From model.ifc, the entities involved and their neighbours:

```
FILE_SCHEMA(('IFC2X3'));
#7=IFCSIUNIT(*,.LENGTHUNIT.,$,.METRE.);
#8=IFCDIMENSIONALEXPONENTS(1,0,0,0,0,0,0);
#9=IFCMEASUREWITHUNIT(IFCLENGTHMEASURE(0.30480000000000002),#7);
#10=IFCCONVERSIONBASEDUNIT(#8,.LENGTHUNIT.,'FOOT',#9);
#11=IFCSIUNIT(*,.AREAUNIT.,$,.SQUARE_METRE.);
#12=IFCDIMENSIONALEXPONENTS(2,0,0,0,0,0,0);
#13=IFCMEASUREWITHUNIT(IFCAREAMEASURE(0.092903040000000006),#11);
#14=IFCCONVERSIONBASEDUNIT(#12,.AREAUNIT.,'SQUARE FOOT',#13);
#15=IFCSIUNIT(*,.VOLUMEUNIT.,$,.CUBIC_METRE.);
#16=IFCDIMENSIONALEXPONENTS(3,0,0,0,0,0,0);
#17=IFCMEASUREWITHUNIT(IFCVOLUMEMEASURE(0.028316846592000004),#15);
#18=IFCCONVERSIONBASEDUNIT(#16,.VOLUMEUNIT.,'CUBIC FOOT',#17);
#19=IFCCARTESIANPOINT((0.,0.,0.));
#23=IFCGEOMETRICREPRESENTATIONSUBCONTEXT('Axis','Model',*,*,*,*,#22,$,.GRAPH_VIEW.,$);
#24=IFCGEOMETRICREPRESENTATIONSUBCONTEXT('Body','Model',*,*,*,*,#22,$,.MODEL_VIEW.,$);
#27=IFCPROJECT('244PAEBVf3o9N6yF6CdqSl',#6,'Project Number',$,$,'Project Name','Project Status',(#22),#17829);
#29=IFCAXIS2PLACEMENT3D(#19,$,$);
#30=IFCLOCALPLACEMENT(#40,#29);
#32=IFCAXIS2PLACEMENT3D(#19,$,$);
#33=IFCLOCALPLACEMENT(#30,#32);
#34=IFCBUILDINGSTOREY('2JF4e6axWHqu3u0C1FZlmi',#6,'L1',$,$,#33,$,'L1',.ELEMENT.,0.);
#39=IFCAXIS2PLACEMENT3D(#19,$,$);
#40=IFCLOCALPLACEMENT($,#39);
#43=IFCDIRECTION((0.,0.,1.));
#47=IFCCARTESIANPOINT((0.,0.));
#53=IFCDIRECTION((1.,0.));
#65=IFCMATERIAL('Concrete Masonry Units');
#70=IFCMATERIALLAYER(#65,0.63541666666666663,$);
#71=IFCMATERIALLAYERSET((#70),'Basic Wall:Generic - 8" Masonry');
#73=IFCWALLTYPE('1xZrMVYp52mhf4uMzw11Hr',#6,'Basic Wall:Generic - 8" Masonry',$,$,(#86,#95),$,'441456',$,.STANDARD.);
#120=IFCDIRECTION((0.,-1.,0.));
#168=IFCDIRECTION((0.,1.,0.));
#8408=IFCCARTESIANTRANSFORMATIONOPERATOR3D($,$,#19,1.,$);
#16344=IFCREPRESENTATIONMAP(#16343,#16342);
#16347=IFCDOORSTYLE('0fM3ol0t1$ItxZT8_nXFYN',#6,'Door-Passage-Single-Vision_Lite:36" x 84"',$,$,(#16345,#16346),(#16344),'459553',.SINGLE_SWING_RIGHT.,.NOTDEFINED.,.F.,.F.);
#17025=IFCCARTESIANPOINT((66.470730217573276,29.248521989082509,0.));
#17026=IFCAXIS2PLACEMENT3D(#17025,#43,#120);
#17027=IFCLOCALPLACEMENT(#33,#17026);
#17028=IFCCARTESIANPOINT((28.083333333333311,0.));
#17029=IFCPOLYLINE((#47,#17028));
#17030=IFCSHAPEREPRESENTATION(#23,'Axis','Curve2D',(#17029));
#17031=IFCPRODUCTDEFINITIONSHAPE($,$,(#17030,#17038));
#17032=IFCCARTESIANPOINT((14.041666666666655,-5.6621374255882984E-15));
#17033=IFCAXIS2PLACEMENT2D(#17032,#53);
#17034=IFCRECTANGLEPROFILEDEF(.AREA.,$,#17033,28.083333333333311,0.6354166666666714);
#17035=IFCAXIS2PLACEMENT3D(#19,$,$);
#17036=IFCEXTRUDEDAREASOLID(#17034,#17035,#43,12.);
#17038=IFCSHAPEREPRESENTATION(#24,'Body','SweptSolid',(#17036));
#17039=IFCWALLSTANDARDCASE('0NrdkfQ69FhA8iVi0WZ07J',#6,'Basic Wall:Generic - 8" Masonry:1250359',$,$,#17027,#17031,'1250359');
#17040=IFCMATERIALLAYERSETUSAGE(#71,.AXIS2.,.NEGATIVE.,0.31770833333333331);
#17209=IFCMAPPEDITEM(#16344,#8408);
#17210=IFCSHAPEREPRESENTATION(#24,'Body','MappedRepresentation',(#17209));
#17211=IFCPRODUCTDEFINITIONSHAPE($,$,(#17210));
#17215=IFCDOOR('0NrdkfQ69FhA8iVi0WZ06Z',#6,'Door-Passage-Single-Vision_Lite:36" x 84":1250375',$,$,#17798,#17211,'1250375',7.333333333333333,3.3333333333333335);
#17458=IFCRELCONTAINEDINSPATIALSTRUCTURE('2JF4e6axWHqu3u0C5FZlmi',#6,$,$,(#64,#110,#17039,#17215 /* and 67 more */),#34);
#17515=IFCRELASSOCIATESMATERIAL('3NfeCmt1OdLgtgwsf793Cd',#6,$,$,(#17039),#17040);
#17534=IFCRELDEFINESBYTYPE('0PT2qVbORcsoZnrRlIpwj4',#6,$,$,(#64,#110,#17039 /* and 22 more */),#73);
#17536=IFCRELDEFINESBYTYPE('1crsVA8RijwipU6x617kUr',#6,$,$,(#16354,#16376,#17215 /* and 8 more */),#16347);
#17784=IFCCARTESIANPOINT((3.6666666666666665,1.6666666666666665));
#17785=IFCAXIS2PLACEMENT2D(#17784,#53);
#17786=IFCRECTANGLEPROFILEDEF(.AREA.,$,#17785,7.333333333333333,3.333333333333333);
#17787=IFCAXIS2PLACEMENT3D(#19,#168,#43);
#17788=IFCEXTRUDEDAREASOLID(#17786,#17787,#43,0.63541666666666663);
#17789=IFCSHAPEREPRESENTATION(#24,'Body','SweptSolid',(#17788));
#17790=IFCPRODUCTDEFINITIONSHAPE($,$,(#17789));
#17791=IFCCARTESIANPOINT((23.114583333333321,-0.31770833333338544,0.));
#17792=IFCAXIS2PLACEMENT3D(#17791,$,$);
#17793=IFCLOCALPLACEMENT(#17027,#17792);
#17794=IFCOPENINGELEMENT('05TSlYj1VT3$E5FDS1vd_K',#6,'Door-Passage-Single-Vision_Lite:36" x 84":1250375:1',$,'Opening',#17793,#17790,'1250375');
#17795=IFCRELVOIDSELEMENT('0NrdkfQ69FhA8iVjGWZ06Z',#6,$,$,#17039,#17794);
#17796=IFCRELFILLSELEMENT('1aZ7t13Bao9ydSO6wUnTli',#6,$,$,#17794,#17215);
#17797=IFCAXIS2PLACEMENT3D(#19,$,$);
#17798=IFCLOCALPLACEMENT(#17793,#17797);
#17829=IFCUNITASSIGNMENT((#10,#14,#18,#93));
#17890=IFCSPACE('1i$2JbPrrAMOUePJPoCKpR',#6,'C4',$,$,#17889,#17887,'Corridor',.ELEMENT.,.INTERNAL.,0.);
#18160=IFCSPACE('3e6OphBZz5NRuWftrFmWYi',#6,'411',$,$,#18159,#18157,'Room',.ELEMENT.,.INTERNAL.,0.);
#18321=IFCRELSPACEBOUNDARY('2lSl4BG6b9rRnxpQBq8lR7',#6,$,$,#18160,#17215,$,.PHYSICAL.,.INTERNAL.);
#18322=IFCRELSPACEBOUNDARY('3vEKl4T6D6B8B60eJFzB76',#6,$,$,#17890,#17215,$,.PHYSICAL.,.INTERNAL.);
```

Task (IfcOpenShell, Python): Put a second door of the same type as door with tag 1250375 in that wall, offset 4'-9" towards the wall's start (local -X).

```python
import ifcopenshell
import ifcopenshell.api.feature
import ifcopenshell.api.geometry
import ifcopenshell.api.root
import ifcopenshell.geom
import ifcopenshell.util.element
import ifcopenshell.util.placement
import ifcopenshell.util.shape
import ifcopenshell.util.unit

model = ifcopenshell.open("model.ifc")
unit_scale = ifcopenshell.util.unit.calculate_unit_scale(model)
settings = ifcopenshell.geom.settings()


def volume(element):
    """Net volume in cubic metres, openings subtracted."""
    shape = ifcopenshell.geom.create_shape(settings, element)
    return ifcopenshell.util.shape.get_volume(shape.geometry)


def reuse_history(source, copy):
    """copy_class also copies each property set's owner history, people and application; keep the originals."""
    for rel in copy.IsDefinedBy:
        if rel.is_a("IfcRelDefinesByProperties") and (history := rel.RelatingPropertyDefinition.OwnerHistory):
            rel.RelatingPropertyDefinition.OwnerHistory = source.OwnerHistory
            ifcopenshell.util.element.remove_deep2(model, history)


door = model.by_guid("0NrdkfQ69FhA8iVi0WZ06Z")
opening = door.FillsVoids[0].RelatingOpeningElement
wall = opening.VoidsElements[0].RelatingBuildingElement
before = volume(wall)
shift = ifcopenshell.util.placement.get_local_placement(wall.ObjectPlacement)[:3, 0] * -57 * 0.0254 / unit_scale

# copy_class copies the void relationship, type, container and properties, but no geometry.
new_opening = ifcopenshell.api.root.copy_class(model, product=opening)
new_opening.Representation = ifcopenshell.util.element.copy_deep(
    model, opening.Representation, exclude=["IfcGeometricRepresentationContext", "IfcRepresentationMap"]
)
new_opening.Name = 'Door-Passage-Single-Vision_Lite:36" x 84"'
new_opening.Tag = None
new_door = ifcopenshell.api.root.copy_class(model, product=door)
new_door.Representation = ifcopenshell.util.element.copy_deep(
    model, door.Representation, exclude=["IfcGeometricRepresentationContext", "IfcRepresentationMap"]
)
new_door.Name = 'Door-Passage-Single-Vision_Lite:36" x 84"'
new_door.Tag = None
reuse_history(door, new_door)
fills = ifcopenshell.api.feature.add_filling(model, opening=new_opening, element=new_door)
fills.OwnerHistory = new_door.OwnerHistory  # required in IFC2X3

for old, new in ((opening, new_opening), (door, new_door)):
    matrix = ifcopenshell.util.placement.get_local_placement(old.ObjectPlacement)
    matrix[:3, 3] += shift
    ifcopenshell.api.geometry.edit_object_placement(model, product=new, matrix=matrix, is_si=False)

after = volume(wall)

print(f"wall volume {before:.3f} -> {after:.3f} m3")

model.write("model_updated.ifc")
```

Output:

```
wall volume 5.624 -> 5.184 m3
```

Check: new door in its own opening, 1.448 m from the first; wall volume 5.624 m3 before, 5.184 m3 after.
